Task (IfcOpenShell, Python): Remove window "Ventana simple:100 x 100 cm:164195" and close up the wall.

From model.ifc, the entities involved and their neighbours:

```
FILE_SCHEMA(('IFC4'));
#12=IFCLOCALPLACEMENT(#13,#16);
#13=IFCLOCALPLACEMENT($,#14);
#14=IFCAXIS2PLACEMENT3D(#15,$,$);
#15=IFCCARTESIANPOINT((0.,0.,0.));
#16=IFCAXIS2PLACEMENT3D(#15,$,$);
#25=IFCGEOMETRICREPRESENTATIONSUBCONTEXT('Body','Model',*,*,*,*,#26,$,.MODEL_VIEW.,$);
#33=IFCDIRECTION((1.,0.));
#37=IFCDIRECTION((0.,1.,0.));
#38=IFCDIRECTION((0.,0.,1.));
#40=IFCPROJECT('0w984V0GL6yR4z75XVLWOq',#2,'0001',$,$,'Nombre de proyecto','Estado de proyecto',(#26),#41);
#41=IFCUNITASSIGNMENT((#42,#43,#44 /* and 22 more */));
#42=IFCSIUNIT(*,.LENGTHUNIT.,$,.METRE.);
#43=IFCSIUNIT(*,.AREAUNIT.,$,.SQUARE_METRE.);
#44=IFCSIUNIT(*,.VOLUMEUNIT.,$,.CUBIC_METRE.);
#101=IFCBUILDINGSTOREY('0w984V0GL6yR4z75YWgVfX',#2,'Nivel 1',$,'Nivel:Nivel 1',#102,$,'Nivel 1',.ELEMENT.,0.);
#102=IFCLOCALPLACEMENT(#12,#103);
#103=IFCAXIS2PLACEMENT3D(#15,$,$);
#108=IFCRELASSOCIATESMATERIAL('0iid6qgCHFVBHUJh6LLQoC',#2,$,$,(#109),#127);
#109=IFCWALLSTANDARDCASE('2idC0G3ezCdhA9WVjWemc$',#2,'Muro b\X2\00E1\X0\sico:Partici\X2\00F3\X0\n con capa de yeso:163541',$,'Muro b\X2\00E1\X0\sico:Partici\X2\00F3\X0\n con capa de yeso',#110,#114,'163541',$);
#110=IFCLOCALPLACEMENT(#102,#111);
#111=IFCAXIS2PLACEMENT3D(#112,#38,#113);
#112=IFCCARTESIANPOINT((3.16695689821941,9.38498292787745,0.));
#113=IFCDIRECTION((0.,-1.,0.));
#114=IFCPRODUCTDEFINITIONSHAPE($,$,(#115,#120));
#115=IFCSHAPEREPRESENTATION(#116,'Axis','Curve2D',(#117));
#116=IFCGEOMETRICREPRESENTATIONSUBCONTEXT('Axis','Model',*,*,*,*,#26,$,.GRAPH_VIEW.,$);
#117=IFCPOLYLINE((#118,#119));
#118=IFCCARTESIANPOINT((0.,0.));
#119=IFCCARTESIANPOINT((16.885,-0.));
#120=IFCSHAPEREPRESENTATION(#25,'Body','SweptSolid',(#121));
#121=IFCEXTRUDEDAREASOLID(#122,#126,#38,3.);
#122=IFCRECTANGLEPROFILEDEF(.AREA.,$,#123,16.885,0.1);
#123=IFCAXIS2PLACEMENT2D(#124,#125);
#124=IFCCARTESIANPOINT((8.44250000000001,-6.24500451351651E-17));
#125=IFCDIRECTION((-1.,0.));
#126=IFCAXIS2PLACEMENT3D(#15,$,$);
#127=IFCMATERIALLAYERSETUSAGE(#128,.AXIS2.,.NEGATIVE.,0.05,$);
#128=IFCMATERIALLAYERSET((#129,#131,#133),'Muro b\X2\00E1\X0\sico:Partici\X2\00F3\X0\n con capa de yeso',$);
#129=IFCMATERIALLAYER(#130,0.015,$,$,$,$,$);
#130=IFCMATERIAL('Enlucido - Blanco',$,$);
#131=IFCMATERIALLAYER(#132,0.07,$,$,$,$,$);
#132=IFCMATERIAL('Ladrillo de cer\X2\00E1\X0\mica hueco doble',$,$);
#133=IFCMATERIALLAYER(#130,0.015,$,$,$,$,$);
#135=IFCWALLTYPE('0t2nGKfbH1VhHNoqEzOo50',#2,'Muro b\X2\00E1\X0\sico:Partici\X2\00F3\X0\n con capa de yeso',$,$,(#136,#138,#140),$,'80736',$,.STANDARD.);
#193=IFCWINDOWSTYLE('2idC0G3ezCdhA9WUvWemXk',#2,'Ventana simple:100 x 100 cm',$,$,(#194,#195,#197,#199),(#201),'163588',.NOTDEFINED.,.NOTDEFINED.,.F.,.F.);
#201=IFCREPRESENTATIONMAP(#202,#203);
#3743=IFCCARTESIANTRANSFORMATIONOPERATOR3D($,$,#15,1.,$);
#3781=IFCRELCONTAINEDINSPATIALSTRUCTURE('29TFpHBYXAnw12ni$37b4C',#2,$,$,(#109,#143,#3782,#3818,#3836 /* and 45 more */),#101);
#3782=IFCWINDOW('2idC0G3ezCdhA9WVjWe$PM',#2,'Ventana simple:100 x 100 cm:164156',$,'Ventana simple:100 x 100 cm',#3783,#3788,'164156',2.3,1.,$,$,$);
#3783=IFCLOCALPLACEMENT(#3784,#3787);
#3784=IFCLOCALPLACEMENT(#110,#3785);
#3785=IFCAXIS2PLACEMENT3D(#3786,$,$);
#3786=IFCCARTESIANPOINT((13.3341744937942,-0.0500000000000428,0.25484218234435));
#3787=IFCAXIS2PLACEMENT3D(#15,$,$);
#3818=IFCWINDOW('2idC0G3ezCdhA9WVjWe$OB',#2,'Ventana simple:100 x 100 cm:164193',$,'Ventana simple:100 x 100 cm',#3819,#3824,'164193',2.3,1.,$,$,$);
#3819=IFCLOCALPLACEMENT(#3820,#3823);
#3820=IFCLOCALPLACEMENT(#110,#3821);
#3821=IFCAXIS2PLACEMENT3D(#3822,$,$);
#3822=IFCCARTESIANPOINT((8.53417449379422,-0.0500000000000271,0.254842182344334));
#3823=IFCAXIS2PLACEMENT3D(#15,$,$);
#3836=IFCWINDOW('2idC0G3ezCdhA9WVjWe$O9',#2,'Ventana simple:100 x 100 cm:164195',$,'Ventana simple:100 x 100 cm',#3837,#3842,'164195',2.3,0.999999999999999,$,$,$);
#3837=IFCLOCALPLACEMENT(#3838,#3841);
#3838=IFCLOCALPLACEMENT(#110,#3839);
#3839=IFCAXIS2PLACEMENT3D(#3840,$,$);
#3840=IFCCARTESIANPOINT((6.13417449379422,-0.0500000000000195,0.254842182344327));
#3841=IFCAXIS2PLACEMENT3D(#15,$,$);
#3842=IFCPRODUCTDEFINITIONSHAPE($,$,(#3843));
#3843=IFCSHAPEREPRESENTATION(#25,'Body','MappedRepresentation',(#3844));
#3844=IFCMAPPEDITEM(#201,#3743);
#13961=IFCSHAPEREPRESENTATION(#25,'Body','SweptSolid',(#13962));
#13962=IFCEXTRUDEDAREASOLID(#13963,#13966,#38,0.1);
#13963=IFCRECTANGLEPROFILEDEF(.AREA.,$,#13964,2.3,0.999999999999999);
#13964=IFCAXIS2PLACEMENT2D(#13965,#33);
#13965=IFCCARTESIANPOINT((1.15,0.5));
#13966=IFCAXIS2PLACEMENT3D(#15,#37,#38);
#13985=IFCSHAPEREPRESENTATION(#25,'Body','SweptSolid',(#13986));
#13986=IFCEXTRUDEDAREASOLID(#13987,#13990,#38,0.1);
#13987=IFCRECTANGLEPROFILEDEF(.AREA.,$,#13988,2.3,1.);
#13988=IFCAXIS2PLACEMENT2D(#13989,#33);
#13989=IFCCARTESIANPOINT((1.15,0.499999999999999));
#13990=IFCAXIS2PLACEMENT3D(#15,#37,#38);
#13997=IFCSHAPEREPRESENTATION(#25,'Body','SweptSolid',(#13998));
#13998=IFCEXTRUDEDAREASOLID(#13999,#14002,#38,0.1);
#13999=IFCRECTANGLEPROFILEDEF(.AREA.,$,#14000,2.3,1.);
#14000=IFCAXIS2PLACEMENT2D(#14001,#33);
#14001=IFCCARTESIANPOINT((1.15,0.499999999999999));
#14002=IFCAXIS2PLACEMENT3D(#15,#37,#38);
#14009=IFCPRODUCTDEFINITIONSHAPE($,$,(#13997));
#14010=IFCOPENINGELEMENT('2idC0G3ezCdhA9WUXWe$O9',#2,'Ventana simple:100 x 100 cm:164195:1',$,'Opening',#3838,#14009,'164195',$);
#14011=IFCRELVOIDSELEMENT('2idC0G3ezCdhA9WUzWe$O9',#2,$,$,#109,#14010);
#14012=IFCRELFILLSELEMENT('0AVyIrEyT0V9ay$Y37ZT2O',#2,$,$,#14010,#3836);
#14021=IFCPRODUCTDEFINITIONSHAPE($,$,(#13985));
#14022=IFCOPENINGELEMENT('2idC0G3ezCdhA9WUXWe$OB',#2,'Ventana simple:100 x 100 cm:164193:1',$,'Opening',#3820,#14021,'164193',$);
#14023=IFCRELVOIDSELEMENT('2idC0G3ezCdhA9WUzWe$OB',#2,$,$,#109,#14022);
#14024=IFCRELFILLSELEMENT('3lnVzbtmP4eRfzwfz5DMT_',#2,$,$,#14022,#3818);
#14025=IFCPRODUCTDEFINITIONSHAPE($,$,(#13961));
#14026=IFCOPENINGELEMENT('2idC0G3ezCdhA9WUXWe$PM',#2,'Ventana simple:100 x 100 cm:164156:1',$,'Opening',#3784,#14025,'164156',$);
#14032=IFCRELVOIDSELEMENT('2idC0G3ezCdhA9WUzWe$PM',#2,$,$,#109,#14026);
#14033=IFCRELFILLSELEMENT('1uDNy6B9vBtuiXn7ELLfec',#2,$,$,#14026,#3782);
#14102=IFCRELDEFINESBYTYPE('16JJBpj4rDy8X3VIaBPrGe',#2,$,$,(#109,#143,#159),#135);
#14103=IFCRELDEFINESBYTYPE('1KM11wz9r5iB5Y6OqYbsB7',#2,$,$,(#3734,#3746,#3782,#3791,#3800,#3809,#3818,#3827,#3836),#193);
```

```python
import ifcopenshell
import ifcopenshell.api.feature
import ifcopenshell.api.root
import ifcopenshell.geom
import ifcopenshell.util.shape

model = ifcopenshell.open("model.ifc")
settings = ifcopenshell.geom.settings()


def volume(element):
    """Net volume in cubic metres, openings subtracted."""
    shape = ifcopenshell.geom.create_shape(settings, element)
    return ifcopenshell.util.shape.get_volume(shape.geometry)


window = model.by_guid("2idC0G3ezCdhA9WVjWe$O9")
opening = window.FillsVoids[0].RelatingOpeningElement
wall = opening.VoidsElements[0].RelatingBuildingElement
before = volume(wall)

ifcopenshell.api.root.remove_product(model, product=window)
ifcopenshell.api.feature.remove_feature(model, feature=opening)

after = volume(wall)

print(f"wall volume {before:.3f} -> {after:.3f} m3")

model.write("model_rev.ifc")
```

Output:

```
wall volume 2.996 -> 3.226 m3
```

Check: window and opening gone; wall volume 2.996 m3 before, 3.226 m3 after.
